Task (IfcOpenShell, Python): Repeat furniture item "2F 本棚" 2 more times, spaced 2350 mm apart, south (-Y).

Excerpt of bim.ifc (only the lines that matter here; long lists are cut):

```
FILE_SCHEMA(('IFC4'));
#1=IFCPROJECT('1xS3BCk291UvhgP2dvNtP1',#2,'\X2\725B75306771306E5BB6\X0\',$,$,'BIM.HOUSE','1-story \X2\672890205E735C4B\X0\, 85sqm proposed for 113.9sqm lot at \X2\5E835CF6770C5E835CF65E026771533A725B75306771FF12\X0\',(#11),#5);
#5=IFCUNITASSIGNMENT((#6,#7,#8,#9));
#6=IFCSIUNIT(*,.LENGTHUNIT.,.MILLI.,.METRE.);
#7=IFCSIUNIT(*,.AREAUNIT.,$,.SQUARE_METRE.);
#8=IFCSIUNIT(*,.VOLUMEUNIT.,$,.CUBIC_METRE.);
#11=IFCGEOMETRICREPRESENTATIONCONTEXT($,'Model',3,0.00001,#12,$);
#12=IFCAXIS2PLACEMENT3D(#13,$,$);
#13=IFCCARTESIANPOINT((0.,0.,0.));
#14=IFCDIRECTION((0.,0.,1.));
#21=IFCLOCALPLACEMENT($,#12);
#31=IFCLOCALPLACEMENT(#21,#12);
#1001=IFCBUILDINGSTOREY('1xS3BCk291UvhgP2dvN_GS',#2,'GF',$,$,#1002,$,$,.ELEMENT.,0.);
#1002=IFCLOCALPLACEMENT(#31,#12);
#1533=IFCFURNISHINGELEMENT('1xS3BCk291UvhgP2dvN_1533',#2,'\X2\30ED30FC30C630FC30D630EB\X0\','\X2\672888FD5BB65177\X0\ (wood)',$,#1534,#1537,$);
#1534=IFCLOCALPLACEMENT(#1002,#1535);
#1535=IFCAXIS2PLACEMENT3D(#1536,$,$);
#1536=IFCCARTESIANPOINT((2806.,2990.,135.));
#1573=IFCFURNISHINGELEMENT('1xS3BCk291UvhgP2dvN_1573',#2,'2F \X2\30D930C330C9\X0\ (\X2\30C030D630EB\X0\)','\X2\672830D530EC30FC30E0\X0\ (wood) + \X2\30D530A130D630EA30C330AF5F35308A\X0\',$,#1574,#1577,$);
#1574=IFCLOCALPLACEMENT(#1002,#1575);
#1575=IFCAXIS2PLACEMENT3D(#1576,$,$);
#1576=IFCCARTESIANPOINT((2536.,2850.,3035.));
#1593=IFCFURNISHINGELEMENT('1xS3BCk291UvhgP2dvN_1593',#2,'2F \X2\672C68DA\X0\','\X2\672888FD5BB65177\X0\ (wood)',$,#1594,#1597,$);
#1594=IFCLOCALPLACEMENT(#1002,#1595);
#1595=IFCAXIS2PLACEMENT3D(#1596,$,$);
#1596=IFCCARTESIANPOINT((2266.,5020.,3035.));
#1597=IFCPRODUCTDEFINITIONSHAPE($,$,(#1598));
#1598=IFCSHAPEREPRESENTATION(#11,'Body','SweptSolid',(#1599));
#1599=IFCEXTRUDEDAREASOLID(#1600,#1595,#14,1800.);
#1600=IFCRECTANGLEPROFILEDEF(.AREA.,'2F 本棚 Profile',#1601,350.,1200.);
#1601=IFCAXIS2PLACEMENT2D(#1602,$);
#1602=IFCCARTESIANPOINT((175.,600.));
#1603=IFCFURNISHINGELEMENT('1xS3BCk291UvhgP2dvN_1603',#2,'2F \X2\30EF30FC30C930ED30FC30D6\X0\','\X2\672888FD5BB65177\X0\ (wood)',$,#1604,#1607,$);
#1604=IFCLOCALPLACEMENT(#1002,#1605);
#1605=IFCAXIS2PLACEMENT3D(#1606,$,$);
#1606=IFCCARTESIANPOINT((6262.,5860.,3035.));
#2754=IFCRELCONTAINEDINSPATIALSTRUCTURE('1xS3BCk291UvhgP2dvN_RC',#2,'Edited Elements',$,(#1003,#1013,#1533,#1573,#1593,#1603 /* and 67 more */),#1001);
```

```python
import numpy as np
import ifcopenshell
import ifcopenshell.api.geometry
import ifcopenshell.api.root
import ifcopenshell.util.element
import ifcopenshell.util.placement

model = ifcopenshell.open("bim.ifc")


def reuse_history(source, copy):
    """copy_class also copies each property set's owner history, people and application; keep the originals."""
    for rel in copy.IsDefinedBy:
        if rel.is_a("IfcRelDefinesByProperties") and (history := rel.RelatingPropertyDefinition.OwnerHistory):
            rel.RelatingPropertyDefinition.OwnerHistory = source.OwnerHistory
            ifcopenshell.util.element.remove_deep2(model, history)


source = model.by_guid("1xS3BCk291UvhgP2dvN_1593")
base = ifcopenshell.util.placement.get_local_placement(source.ObjectPlacement)
step = np.array([0.0, -1.0, 0.0]) * 2350.0

for i in range(1, 3):
    copy = ifcopenshell.api.root.copy_class(model, product=source)
    copy.Representation = ifcopenshell.util.element.copy_deep(
        model, source.Representation, exclude=["IfcGeometricRepresentationContext", "IfcRepresentationMap"]
    )
    reuse_history(source, copy)
    matrix = base.copy()
    matrix[:3, 3] += i * step
    print("added at", matrix[:3, 3].round(3) + 0.0)
    ifcopenshell.api.geometry.edit_object_placement(model, product=copy, matrix=matrix, is_si=False)

model.write("bim-out.ifc")
```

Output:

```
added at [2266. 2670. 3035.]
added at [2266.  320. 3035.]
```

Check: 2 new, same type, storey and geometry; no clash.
